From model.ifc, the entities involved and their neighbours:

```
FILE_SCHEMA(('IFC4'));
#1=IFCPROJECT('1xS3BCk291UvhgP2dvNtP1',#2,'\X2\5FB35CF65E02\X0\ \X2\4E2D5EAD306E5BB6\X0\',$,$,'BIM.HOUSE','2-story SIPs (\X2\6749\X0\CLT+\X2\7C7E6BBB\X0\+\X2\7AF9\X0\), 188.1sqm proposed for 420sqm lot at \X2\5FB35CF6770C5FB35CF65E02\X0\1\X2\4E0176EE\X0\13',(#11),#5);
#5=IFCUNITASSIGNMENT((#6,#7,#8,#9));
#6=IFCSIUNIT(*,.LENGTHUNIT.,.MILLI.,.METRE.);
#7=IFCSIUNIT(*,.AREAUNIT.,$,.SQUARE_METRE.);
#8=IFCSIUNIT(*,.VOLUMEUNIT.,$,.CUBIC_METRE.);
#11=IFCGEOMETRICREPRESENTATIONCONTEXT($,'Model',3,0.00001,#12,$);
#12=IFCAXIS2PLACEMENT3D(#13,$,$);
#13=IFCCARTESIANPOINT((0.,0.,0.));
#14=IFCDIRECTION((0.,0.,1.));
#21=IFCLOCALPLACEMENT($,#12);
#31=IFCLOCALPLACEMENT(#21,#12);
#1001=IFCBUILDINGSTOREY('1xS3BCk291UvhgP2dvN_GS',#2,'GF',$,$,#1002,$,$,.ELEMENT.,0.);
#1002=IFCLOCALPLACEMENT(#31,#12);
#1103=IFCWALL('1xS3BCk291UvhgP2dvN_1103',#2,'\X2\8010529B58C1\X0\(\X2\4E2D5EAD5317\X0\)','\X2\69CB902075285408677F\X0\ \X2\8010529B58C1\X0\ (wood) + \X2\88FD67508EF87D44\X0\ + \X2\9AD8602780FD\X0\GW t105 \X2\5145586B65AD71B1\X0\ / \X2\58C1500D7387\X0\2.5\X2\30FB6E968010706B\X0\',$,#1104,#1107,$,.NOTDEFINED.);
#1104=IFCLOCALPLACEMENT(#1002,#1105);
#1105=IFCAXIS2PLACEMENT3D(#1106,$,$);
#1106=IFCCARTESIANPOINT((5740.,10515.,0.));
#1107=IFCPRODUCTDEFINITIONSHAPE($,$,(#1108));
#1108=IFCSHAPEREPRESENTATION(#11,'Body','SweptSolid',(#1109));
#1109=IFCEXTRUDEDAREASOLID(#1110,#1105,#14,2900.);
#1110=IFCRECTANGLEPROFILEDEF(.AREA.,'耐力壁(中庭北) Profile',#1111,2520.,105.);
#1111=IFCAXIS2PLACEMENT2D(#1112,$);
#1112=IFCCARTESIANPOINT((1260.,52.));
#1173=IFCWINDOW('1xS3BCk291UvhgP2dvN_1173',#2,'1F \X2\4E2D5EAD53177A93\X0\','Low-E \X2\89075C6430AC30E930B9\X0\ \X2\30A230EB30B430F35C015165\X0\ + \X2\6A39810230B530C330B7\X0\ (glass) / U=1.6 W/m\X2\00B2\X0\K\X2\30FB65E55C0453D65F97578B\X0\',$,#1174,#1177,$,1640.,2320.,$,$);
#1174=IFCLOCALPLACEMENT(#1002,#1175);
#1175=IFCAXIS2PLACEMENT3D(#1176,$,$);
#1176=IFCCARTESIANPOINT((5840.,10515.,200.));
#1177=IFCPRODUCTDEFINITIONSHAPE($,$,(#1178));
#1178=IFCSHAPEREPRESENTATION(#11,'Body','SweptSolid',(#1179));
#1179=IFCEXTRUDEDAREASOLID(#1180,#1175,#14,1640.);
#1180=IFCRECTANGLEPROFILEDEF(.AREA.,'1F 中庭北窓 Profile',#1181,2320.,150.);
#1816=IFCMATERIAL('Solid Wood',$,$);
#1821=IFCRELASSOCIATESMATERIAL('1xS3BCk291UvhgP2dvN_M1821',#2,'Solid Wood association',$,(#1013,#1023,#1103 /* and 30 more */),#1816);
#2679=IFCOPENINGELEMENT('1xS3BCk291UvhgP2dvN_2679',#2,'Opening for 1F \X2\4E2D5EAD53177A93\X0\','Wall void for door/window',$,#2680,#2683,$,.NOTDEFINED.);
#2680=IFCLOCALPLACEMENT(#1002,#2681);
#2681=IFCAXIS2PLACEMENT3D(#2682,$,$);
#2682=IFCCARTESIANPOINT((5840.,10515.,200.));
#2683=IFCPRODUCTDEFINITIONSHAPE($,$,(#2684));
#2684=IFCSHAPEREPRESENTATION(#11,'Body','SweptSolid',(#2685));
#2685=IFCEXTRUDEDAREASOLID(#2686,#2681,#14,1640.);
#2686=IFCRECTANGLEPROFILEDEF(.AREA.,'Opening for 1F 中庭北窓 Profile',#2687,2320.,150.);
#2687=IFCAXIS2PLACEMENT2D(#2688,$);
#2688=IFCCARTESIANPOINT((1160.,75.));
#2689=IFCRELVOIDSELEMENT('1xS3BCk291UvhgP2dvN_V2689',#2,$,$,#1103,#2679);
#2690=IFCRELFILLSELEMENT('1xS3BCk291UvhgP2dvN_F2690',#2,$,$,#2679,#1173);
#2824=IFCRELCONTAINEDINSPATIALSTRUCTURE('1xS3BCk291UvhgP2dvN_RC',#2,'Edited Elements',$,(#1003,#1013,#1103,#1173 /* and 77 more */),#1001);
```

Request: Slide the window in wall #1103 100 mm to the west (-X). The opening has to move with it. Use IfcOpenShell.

```python
import ifcopenshell
import ifcopenshell.api.geometry
import ifcopenshell.util.placement
import ifcopenshell.util.unit

model = ifcopenshell.open("model.ifc")
unit_scale = ifcopenshell.util.unit.calculate_unit_scale(model)

window = model.by_guid("1xS3BCk291UvhgP2dvN_1173")
opening = window.FillsVoids[0].RelatingOpeningElement
wall = opening.VoidsElements[0].RelatingBuildingElement

wall_matrix = ifcopenshell.util.placement.get_local_placement(wall.ObjectPlacement)
shift = wall_matrix[:3, 0] * -0.1 / unit_scale
before = ifcopenshell.util.placement.get_local_placement(window.ObjectPlacement)[:3, 3].copy()

# The window is not placed relative to its opening, so move both.
for product in (opening, window):
    matrix = ifcopenshell.util.placement.get_local_placement(product.ObjectPlacement)
    matrix[:3, 3] += shift
    ifcopenshell.api.geometry.edit_object_placement(model, product=product, matrix=matrix, is_si=False)

after = ifcopenshell.util.placement.get_local_placement(window.ObjectPlacement)[:3, 3]
print("window moved by", (after - before).round(3) + 0.0)

model.write("model_edited.ifc")
```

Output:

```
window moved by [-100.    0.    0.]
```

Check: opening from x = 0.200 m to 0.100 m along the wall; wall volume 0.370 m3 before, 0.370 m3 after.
